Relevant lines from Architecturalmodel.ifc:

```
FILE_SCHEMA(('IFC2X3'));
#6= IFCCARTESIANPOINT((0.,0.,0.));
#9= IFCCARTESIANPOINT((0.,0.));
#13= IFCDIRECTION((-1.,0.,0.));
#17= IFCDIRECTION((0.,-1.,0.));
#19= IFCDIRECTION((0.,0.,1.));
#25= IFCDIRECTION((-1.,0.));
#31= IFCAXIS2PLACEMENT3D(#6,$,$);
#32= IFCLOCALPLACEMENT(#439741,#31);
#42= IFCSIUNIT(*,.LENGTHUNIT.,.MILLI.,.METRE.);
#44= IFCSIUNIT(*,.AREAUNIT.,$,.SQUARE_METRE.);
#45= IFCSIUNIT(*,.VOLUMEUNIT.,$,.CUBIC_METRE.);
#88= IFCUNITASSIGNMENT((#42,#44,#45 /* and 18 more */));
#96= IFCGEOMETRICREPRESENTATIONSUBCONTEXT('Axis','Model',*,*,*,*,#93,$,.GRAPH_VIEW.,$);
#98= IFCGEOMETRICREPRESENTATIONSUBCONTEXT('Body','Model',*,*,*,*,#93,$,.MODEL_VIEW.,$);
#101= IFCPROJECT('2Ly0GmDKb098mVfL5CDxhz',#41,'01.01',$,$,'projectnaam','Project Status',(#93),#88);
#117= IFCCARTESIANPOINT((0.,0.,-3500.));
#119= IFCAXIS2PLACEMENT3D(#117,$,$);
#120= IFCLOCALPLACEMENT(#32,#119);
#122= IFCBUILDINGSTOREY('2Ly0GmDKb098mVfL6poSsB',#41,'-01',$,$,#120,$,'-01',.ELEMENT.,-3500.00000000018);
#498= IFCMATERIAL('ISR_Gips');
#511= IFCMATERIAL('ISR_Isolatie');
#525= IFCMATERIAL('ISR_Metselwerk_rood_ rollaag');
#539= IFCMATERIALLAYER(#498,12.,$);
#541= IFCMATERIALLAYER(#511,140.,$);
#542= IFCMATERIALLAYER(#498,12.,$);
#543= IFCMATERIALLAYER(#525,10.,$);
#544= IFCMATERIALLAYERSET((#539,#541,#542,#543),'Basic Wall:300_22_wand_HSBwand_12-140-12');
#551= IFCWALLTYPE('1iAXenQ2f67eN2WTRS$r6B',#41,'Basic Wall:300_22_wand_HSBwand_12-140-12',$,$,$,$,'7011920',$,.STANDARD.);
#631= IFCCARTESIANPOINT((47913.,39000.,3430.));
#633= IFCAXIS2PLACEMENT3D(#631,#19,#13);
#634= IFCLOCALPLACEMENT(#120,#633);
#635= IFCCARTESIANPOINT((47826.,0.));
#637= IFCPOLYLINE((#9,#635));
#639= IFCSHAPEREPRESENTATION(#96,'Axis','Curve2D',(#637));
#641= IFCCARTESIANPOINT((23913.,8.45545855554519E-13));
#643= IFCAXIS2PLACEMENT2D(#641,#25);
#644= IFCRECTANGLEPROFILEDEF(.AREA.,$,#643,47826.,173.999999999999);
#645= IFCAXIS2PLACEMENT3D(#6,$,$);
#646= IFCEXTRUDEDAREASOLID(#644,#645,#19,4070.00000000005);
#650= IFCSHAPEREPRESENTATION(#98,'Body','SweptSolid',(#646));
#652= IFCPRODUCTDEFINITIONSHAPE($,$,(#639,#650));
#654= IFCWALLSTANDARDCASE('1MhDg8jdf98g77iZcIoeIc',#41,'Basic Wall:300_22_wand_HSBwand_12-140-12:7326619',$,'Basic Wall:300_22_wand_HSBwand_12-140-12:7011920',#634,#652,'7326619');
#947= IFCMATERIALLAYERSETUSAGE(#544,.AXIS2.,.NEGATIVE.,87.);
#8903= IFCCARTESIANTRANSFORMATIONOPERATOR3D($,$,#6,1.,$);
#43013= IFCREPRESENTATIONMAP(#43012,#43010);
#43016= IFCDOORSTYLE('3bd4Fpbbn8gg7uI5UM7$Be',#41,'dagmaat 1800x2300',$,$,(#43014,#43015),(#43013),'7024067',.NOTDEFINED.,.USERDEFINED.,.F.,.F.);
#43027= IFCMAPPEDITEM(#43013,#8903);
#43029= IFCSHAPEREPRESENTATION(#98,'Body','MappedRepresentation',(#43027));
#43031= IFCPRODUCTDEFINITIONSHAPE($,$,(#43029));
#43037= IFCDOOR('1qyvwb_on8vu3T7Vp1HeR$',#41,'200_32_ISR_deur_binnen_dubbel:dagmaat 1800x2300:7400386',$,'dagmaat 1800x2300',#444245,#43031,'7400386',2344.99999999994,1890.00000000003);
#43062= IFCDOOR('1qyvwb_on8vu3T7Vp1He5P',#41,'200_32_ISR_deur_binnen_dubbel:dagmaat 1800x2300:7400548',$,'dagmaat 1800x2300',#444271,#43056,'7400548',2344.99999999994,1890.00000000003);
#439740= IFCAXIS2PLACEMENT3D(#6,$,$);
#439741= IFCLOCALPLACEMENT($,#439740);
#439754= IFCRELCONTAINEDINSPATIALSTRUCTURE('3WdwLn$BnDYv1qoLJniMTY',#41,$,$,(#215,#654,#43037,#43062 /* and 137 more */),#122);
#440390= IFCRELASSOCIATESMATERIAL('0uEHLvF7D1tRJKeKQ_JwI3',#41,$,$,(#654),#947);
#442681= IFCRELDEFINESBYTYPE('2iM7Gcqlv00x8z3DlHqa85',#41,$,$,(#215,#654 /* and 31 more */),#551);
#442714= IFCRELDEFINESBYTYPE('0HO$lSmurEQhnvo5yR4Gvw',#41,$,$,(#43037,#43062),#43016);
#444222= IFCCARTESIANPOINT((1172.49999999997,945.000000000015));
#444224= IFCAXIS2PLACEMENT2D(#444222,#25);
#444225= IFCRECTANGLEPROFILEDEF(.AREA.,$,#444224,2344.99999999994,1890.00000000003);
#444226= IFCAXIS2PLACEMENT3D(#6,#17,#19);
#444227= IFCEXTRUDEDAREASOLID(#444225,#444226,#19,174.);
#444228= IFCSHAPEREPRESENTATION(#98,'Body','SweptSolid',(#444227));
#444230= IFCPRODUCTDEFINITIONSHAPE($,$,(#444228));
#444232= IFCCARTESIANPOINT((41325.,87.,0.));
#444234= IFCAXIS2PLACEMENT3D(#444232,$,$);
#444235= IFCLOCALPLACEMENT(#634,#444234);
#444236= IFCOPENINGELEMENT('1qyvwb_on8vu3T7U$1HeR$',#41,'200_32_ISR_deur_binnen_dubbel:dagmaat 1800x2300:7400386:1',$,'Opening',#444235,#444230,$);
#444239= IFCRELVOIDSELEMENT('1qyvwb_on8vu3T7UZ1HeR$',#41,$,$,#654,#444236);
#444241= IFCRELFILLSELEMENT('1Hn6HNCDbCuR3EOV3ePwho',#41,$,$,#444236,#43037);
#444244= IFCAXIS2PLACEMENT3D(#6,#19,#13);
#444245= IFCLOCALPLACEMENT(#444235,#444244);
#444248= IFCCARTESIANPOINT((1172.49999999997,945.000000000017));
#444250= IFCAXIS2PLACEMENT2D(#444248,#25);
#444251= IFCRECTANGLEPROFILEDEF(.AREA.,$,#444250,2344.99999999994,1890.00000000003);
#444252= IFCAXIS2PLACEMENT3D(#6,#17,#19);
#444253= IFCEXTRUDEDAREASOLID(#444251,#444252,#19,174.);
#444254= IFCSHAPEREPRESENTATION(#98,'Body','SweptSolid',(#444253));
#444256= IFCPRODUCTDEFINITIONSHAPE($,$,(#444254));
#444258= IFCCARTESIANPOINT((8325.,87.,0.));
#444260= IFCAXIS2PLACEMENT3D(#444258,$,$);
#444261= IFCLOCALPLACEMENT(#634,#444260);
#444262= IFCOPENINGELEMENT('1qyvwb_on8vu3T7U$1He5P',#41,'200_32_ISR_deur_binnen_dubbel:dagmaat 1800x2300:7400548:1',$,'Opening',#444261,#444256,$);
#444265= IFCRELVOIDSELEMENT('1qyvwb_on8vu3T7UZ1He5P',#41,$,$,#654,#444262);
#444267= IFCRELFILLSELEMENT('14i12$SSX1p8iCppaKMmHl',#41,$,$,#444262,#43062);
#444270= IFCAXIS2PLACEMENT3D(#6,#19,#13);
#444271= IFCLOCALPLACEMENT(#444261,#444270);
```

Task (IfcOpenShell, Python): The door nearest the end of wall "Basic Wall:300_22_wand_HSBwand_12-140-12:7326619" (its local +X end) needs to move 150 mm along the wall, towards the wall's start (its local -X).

```python
import ifcopenshell
import ifcopenshell.api.geometry
import ifcopenshell.util.placement

model = ifcopenshell.open("Architecturalmodel.ifc")

door = model.by_id(43037)
opening = door.FillsVoids[0].RelatingOpeningElement
wall = opening.VoidsElements[0].RelatingBuildingElement

wall_matrix = ifcopenshell.util.placement.get_local_placement(wall.ObjectPlacement)
shift = wall_matrix[:3, 0] * -150.0
before = ifcopenshell.util.placement.get_local_placement(door.ObjectPlacement)[:3, 3].copy()

# The door is placed relative to its opening, so it follows when the opening moves.
matrix = ifcopenshell.util.placement.get_local_placement(opening.ObjectPlacement)
matrix[:3, 3] += shift
ifcopenshell.api.geometry.edit_object_placement(
    model, product=opening, matrix=matrix, is_si=False, should_transform_children=True
)

after = ifcopenshell.util.placement.get_local_placement(door.ObjectPlacement)[:3, 3]
print("door moved by", (after - before).round(3) + 0.0)

model.write("Architecturalmodel_updated.ifc")
```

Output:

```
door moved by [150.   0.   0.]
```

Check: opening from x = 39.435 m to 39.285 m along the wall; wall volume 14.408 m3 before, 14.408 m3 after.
